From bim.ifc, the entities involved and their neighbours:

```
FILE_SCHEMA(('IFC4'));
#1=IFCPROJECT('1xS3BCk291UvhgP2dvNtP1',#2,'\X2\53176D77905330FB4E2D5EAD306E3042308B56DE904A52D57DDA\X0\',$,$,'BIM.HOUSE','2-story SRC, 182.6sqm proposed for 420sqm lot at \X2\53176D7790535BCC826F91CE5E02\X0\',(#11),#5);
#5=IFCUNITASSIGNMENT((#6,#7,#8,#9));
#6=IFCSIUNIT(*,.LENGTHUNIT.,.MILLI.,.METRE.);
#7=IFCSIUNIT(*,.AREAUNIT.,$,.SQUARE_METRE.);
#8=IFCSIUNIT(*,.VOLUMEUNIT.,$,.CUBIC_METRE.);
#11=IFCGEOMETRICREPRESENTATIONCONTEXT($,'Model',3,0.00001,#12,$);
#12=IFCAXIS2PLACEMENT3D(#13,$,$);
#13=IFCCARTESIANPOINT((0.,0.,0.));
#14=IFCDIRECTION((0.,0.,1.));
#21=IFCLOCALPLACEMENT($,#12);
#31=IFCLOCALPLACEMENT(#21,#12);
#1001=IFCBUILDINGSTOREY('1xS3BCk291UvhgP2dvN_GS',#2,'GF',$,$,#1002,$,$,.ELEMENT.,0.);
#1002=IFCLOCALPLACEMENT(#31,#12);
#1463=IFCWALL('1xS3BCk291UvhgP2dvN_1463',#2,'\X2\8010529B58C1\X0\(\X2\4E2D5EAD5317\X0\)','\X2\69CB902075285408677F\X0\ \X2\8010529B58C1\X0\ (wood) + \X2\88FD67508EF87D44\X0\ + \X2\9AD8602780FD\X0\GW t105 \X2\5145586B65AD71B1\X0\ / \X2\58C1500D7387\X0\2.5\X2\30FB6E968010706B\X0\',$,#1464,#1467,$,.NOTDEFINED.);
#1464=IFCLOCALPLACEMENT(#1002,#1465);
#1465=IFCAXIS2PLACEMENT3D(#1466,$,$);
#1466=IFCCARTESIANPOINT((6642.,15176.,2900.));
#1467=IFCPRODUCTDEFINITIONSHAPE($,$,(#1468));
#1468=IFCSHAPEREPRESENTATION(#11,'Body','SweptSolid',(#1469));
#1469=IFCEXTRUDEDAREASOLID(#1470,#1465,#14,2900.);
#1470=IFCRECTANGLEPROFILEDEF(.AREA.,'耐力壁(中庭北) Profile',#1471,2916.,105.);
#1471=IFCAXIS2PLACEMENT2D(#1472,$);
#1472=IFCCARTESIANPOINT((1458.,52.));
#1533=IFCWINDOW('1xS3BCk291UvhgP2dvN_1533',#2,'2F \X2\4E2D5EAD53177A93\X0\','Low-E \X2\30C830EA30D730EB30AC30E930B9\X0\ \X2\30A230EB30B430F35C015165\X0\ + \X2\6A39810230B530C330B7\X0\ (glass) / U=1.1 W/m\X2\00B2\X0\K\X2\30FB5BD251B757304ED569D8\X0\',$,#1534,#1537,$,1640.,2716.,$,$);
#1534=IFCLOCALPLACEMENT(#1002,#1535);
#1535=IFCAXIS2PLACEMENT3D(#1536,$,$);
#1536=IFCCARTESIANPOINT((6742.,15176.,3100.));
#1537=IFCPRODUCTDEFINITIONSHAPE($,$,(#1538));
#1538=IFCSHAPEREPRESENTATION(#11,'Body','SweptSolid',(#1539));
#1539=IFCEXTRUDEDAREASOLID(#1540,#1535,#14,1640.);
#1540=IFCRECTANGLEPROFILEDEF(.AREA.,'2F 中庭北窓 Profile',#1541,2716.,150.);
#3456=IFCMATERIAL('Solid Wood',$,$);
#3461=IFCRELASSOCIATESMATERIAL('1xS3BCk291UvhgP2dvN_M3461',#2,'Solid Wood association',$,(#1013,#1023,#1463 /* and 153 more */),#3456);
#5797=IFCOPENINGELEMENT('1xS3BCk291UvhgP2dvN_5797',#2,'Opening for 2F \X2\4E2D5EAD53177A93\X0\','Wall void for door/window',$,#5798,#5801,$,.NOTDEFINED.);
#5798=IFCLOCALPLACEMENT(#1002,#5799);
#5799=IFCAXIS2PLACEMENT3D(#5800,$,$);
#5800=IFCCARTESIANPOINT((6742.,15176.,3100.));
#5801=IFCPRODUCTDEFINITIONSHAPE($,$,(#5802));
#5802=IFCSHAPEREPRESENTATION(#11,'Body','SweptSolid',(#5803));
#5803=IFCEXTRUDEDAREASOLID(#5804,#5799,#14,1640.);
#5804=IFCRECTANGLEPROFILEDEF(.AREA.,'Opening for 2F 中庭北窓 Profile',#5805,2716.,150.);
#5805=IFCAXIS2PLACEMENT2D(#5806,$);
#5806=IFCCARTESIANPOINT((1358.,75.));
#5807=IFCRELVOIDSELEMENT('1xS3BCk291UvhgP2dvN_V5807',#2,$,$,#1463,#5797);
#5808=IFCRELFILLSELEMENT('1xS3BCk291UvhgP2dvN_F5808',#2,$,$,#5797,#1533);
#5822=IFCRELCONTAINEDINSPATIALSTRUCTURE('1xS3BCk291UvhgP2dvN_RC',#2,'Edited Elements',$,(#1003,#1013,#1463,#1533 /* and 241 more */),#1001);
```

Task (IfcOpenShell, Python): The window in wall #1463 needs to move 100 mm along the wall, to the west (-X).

```python
import ifcopenshell
import ifcopenshell.api.geometry
import ifcopenshell.util.placement
import ifcopenshell.util.unit

model = ifcopenshell.open("bim.ifc")
unit_scale = ifcopenshell.util.unit.calculate_unit_scale(model)

window = model.by_guid("1xS3BCk291UvhgP2dvN_1533")
opening = window.FillsVoids[0].RelatingOpeningElement
wall = opening.VoidsElements[0].RelatingBuildingElement

wall_matrix = ifcopenshell.util.placement.get_local_placement(wall.ObjectPlacement)
shift = wall_matrix[:3, 0] * -0.1 / unit_scale
before = ifcopenshell.util.placement.get_local_placement(window.ObjectPlacement)[:3, 3].copy()

# The window is not placed relative to its opening, so move both.
for product in (opening, window):
    matrix = ifcopenshell.util.placement.get_local_placement(product.ObjectPlacement)
    matrix[:3, 3] += shift
    ifcopenshell.api.geometry.edit_object_placement(model, product=product, matrix=matrix, is_si=False)

after = ifcopenshell.util.placement.get_local_placement(window.ObjectPlacement)[:3, 3]
print("window moved by", (after - before).round(3) + 0.0)

model.write("bim_updated.ifc")
```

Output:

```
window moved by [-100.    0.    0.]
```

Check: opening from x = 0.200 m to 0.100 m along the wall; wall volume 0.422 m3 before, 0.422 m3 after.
